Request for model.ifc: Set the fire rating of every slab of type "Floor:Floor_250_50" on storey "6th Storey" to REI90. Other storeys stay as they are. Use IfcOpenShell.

First a look at what the model holds.

```python
import ifcopenshell
import ifcopenshell.util.element

model = ifcopenshell.open("model.ifc")
print(model.schema)
storey = next(s for s in model.by_type("IfcBuildingStorey") if s.Name == "6th Storey")
slabs = [e for e in ifcopenshell.util.element.get_decomposition(storey) if e.is_a("IfcSlab")]
seen = {}
for e in slabs:
    element_type = ifcopenshell.util.element.get_type(e)
    key = (element_type.Name if element_type != e and element_type else None, ifcopenshell.util.element.get_pset(e, "Pset_SlabCommon", "FireRating"))
    seen[key] = seen.get(key, 0) + 1
for (name, value), count in sorted(seen.items(), key=str):
    print(count, "x", name, "|", value)
```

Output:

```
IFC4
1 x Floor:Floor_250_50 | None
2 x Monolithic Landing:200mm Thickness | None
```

```python
import ifcopenshell
import ifcopenshell.api.pset
import ifcopenshell.util.element

model = ifcopenshell.open("model.ifc")

storey = next(s for s in model.by_type("IfcBuildingStorey") if s.Name == "6th Storey")
slabs = [e for e in ifcopenshell.util.element.get_decomposition(storey) if e.is_a("IfcSlab")]

count = 0
for e in slabs:
    element_type = ifcopenshell.util.element.get_type(e)
    if element_type in (None, e) or element_type.Name != "Floor:Floor_250_50":
        continue
    # add_pset returns the element's existing set when there is one.
    pset = ifcopenshell.api.pset.add_pset(model, product=e, name="Pset_SlabCommon")
    ifcopenshell.api.pset.edit_pset(model, pset=pset, properties={"FireRating": "REI90"})
    count += 1

print(count, "slabs updated")

model.write("model_updated.ifc")
```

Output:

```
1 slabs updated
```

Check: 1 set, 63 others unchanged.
